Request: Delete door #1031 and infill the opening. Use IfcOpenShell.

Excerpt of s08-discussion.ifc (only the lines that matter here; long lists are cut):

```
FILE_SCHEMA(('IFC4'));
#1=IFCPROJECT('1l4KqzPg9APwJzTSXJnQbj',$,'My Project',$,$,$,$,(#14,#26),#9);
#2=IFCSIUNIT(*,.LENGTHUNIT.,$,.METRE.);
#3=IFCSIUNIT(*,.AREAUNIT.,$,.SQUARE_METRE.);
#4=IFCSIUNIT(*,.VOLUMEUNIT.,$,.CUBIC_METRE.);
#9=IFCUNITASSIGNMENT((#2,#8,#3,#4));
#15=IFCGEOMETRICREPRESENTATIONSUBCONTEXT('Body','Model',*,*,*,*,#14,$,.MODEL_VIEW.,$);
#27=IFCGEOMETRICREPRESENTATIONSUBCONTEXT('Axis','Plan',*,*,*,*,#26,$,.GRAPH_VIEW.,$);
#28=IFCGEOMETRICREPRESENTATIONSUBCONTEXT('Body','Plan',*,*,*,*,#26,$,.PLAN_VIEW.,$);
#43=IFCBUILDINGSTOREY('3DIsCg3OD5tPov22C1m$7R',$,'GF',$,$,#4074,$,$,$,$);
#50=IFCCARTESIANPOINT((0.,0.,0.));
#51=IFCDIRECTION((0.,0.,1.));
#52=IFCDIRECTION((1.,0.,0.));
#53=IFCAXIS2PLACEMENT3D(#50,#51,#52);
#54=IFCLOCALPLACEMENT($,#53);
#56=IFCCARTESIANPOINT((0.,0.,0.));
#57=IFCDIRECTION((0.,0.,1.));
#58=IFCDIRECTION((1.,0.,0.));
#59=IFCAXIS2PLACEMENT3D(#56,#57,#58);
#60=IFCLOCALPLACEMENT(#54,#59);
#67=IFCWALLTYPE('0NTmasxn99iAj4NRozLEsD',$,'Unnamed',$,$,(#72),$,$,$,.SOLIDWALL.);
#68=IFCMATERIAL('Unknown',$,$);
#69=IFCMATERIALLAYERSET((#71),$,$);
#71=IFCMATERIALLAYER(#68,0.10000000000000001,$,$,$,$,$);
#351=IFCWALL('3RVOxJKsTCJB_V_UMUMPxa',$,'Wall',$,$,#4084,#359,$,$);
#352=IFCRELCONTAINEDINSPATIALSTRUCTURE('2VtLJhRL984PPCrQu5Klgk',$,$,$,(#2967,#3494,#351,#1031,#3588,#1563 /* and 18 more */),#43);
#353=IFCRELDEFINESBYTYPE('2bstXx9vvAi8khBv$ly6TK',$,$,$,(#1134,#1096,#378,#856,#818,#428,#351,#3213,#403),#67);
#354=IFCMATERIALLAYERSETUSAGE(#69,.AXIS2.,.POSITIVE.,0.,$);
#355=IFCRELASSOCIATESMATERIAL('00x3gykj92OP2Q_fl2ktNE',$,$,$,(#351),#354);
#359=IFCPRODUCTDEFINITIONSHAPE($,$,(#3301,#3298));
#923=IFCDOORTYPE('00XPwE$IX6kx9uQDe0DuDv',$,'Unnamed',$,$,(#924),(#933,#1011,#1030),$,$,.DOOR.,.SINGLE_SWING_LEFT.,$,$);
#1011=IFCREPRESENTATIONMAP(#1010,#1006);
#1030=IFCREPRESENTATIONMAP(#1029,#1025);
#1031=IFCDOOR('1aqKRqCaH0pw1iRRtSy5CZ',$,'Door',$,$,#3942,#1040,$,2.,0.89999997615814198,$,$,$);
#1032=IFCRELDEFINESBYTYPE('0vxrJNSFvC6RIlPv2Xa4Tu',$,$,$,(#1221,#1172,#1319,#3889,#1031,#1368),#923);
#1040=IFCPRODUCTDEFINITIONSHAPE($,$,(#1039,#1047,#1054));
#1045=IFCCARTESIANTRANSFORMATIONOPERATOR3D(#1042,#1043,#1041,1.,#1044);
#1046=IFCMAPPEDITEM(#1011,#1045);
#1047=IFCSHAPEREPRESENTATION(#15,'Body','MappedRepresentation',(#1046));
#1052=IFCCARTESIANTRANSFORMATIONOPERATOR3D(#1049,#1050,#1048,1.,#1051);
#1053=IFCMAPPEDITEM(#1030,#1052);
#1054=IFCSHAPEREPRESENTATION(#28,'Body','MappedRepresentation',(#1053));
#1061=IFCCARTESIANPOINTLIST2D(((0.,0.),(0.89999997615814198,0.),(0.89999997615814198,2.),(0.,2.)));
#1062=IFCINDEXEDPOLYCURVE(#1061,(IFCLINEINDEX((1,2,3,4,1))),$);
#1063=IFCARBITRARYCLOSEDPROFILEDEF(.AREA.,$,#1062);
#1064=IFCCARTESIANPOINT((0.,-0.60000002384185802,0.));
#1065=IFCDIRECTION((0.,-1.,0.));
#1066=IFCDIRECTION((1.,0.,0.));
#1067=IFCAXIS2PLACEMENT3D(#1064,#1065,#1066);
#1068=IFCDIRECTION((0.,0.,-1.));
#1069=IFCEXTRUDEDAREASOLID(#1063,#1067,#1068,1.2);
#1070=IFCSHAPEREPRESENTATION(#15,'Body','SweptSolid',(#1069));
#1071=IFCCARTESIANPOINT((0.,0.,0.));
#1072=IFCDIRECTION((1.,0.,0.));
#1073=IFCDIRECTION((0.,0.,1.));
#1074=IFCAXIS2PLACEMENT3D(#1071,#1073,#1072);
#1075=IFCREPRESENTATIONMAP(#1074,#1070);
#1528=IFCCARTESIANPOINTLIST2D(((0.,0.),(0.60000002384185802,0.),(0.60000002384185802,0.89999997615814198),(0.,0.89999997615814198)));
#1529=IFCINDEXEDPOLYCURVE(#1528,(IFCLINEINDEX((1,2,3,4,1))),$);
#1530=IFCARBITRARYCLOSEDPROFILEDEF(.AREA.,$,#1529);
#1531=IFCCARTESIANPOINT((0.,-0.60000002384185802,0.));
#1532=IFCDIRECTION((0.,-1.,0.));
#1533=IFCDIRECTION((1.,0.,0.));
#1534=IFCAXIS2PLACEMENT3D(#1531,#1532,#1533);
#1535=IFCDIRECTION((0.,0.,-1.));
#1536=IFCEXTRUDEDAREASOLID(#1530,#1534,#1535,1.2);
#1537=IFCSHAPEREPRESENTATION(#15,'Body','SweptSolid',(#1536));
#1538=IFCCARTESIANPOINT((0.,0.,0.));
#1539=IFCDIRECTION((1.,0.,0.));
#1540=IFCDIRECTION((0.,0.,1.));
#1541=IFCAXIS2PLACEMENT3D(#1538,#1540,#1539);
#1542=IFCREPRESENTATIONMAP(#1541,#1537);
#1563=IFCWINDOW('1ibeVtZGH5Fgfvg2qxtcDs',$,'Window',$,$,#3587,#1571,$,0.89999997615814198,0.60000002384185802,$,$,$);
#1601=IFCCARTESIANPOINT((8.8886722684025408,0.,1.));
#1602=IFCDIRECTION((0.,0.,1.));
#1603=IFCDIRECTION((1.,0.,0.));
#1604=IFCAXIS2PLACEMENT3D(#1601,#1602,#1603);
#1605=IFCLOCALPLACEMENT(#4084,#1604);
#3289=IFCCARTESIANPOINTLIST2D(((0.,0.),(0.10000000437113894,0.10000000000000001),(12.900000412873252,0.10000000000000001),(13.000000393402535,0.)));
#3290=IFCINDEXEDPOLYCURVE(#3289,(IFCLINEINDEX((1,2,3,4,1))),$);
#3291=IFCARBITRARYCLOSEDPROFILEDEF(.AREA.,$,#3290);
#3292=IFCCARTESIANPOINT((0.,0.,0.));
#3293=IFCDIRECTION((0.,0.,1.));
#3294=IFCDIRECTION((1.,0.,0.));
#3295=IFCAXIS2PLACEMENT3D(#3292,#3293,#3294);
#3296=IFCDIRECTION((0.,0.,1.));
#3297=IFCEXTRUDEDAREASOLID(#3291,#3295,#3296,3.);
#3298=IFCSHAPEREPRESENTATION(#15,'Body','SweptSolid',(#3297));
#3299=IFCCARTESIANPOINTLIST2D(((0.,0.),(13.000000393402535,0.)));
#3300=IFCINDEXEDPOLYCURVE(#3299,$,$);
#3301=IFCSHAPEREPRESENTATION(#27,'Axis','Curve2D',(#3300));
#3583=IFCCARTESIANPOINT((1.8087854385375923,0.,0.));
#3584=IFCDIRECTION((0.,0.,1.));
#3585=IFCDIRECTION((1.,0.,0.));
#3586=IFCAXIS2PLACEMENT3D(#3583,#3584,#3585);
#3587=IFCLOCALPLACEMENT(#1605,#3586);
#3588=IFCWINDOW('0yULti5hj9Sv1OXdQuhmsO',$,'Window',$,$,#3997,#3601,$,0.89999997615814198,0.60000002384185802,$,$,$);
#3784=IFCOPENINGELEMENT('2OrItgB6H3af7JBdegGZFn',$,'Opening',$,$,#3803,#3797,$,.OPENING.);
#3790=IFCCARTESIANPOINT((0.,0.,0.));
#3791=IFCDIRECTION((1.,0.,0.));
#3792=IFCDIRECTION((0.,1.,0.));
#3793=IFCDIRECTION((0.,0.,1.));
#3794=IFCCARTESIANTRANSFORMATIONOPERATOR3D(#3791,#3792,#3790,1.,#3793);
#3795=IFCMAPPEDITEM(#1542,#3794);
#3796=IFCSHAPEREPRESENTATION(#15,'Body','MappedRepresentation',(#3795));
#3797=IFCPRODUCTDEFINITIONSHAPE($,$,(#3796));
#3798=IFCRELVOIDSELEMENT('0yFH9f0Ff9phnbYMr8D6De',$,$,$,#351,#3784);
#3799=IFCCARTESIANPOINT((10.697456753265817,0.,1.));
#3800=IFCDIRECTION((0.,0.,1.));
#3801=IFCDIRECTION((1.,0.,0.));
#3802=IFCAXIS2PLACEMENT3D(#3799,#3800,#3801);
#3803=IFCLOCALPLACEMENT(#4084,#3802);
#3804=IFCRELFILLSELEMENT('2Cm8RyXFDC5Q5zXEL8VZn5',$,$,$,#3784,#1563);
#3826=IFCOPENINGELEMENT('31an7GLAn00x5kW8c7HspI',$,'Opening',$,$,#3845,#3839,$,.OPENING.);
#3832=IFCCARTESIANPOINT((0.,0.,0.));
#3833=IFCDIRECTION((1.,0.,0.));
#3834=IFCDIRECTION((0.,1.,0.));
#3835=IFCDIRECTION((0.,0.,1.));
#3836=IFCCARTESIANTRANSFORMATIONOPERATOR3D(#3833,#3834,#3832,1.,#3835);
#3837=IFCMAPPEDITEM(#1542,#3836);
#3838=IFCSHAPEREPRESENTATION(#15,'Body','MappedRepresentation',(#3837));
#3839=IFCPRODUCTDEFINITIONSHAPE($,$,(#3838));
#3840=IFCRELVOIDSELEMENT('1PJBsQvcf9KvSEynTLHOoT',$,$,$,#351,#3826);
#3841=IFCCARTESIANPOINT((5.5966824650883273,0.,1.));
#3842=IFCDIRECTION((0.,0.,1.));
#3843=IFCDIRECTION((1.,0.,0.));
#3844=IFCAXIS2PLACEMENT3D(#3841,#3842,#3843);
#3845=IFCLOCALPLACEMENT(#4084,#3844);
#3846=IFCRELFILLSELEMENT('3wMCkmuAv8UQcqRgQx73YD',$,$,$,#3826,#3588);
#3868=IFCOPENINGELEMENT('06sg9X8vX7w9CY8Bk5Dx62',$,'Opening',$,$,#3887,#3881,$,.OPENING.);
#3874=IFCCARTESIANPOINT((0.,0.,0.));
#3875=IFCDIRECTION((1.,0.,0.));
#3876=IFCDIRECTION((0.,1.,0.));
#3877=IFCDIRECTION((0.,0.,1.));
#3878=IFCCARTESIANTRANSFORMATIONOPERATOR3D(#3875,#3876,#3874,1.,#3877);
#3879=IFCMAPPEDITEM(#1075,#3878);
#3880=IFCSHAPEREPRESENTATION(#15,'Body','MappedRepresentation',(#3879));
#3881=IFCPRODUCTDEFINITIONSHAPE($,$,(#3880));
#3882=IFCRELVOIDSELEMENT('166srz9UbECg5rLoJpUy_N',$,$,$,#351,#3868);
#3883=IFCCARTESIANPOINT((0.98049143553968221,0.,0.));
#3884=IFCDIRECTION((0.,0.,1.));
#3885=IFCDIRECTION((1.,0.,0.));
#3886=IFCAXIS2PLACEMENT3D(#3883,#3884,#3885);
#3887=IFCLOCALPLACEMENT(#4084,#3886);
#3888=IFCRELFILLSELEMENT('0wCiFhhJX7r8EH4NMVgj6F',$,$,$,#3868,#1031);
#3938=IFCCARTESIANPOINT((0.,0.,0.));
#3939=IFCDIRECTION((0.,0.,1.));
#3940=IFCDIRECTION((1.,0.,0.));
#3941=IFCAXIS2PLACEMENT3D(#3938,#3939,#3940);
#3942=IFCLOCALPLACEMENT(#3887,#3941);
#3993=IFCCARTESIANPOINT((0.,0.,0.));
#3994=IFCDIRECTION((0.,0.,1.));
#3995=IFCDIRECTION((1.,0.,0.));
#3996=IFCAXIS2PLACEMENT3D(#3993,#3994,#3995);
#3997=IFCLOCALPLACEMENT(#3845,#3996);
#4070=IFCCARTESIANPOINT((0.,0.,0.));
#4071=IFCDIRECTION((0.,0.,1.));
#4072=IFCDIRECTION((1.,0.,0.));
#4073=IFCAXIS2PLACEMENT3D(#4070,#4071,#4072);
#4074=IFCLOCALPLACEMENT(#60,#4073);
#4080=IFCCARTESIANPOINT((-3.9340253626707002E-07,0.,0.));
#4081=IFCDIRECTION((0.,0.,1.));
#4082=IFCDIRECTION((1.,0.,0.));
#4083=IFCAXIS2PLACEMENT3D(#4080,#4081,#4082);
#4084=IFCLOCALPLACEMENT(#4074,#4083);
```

```python
import ifcopenshell
import ifcopenshell.api.feature
import ifcopenshell.api.root
import ifcopenshell.geom
import ifcopenshell.util.shape

model = ifcopenshell.open("s08-discussion.ifc")
settings = ifcopenshell.geom.settings()


def volume(element):
    """Net volume in cubic metres, openings subtracted."""
    shape = ifcopenshell.geom.create_shape(settings, element)
    return ifcopenshell.util.shape.get_volume(shape.geometry)


door = model.by_guid("1aqKRqCaH0pw1iRRtSy5CZ")
opening = door.FillsVoids[0].RelatingOpeningElement
wall = opening.VoidsElements[0].RelatingBuildingElement
before = volume(wall)

ifcopenshell.api.root.remove_product(model, product=door)
ifcopenshell.api.feature.remove_feature(model, feature=opening)

after = volume(wall)

print(f"wall volume {before:.3f} -> {after:.3f} m3")

model.write("s08-discussion_v2.ifc")
```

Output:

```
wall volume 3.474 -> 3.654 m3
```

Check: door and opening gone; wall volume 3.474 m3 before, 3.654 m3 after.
